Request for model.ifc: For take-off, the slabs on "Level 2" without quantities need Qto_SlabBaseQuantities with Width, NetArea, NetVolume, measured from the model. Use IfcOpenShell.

First a look at what the model holds.

```python
import ifcopenshell
import ifcopenshell.util.element
import ifcopenshell.util.unit

model = ifcopenshell.open("model.ifc")
print(model.schema)
for unit_type in ("LENGTHUNIT", "AREAUNIT", "VOLUMEUNIT"):
    print(unit_type, ifcopenshell.util.unit.calculate_unit_scale(model, unit_type))
storey = next(s for s in model.by_type("IfcBuildingStorey") if s.Name == "Level 2")
slabs = [e for e in ifcopenshell.util.element.get_decomposition(storey) if e.is_a("IfcSlab")]
for e in sorted(slabs, key=lambda e: e.id()):
    print(e.id(), e.is_a(), e.Name, list(ifcopenshell.util.element.get_psets(e, qtos_only=True)), sep=" | ")
```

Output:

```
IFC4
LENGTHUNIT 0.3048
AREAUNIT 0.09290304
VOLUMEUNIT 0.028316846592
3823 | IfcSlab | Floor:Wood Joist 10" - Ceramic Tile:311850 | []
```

```python
import ifcopenshell
import ifcopenshell.api.pset
import ifcopenshell.geom
import ifcopenshell.util.element
import ifcopenshell.util.shape
import ifcopenshell.util.unit

model = ifcopenshell.open("model.ifc")
unit_scale = ifcopenshell.util.unit.calculate_unit_scale(model)
area_scale = ifcopenshell.util.unit.calculate_unit_scale(model, "AREAUNIT")
volume_scale = ifcopenshell.util.unit.calculate_unit_scale(model, "VOLUMEUNIT")
settings = ifcopenshell.geom.settings()

storey = next(s for s in model.by_type("IfcBuildingStorey") if s.Name == "Level 2")
slabs = [e for e in ifcopenshell.util.element.get_decomposition(storey) if e.is_a("IfcSlab")]

for e in sorted(slabs, key=lambda e: e.id()):
    if ifcopenshell.util.element.get_psets(e, qtos_only=True, should_inherit=False):
        continue
    # Geometry comes back in metres, in the element's own axes.
    shape = ifcopenshell.geom.create_shape(settings, e)
    values = {
        "Width": ifcopenshell.util.shape.get_z(shape.geometry) / unit_scale,
        "NetArea": ifcopenshell.util.shape.get_footprint_area(shape.geometry) / area_scale,
        "NetVolume": ifcopenshell.util.shape.get_volume(shape.geometry) / volume_scale,
    }
    qto = ifcopenshell.api.pset.add_qto(model, product=e, name="Qto_SlabBaseQuantities")
    ifcopenshell.api.pset.edit_qto(model, qto=qto, properties=values)
    print(e.id(), {k: round(v, 3) for k, v in values.items()})

model.write("model_updated.ifc")
```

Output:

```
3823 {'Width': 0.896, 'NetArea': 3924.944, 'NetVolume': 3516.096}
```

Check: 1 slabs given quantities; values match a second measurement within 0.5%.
